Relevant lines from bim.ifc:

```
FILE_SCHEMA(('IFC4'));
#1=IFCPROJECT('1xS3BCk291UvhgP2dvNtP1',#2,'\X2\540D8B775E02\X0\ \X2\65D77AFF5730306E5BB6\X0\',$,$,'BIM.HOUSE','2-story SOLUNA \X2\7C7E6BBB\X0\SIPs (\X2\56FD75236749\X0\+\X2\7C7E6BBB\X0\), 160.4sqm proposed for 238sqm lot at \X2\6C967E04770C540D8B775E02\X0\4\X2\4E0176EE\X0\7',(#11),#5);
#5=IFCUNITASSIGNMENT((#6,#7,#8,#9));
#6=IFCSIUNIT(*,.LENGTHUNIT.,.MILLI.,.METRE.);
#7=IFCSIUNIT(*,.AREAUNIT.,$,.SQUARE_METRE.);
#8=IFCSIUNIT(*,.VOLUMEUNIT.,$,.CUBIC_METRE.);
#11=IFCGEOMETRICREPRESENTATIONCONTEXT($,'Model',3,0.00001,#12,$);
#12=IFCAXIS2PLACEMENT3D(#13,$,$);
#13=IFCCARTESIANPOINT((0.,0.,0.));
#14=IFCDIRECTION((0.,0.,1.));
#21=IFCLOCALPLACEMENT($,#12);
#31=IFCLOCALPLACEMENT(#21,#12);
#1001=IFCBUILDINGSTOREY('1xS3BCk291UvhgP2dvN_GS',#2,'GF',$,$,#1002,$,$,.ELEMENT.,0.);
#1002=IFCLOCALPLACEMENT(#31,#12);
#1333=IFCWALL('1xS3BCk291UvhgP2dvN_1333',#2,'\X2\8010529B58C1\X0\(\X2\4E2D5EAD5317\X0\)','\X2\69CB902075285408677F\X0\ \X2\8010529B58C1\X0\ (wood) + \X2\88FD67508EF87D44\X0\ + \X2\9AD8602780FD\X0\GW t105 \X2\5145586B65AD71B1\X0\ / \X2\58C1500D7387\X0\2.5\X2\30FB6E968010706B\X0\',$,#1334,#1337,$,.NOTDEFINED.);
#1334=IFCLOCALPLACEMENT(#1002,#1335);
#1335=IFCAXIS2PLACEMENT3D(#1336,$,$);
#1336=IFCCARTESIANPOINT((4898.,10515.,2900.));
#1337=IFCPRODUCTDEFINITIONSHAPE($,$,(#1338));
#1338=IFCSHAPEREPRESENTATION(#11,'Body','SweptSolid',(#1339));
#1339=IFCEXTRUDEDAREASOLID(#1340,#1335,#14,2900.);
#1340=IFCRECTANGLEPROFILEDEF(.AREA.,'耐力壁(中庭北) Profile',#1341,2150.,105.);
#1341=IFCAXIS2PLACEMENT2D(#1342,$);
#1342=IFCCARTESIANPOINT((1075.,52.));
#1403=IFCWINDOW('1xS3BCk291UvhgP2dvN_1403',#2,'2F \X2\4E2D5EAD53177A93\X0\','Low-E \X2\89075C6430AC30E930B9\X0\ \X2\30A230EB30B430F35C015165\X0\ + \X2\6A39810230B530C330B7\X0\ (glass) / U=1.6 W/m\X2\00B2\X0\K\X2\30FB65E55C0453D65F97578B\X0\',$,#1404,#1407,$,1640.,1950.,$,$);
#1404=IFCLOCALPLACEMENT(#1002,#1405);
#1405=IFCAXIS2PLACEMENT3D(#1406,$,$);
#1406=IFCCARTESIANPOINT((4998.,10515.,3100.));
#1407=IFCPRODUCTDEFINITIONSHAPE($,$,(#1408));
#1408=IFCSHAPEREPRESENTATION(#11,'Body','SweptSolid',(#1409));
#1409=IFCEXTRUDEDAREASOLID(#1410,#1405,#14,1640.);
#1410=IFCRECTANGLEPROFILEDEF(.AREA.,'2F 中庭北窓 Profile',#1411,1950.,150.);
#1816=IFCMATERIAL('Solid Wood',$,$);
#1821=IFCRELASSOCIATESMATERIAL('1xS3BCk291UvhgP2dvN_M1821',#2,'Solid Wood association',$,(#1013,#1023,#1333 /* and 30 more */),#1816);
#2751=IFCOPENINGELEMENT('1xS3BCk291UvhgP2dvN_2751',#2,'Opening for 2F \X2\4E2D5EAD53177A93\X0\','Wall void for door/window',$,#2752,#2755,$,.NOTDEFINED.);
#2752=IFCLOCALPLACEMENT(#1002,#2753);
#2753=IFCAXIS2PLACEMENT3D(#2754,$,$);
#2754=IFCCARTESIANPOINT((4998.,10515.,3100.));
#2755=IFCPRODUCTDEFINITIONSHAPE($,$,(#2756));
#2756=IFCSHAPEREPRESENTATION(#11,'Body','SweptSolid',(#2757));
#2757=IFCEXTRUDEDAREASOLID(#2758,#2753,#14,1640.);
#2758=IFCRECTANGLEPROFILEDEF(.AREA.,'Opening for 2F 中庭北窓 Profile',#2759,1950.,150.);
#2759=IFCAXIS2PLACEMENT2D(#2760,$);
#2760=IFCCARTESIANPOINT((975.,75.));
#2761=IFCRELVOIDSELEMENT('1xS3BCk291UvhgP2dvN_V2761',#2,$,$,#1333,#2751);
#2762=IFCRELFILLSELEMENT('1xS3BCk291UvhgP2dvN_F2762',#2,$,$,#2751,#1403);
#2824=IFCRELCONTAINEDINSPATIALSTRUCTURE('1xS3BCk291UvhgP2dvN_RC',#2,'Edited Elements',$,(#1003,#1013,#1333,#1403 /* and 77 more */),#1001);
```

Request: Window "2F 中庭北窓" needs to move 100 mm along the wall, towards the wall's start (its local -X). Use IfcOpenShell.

```python
import ifcopenshell
import ifcopenshell.api.geometry
import ifcopenshell.util.placement
import ifcopenshell.util.unit

model = ifcopenshell.open("bim.ifc")
unit_scale = ifcopenshell.util.unit.calculate_unit_scale(model)

window = model.by_guid("1xS3BCk291UvhgP2dvN_1403")
opening = window.FillsVoids[0].RelatingOpeningElement
wall = opening.VoidsElements[0].RelatingBuildingElement

wall_matrix = ifcopenshell.util.placement.get_local_placement(wall.ObjectPlacement)
shift = wall_matrix[:3, 0] * -0.1 / unit_scale
before = ifcopenshell.util.placement.get_local_placement(window.ObjectPlacement)[:3, 3].copy()

# The window is not placed relative to its opening, so move both.
for product in (opening, window):
    matrix = ifcopenshell.util.placement.get_local_placement(product.ObjectPlacement)
    matrix[:3, 3] += shift
    ifcopenshell.api.geometry.edit_object_placement(model, product=product, matrix=matrix, is_si=False)

after = ifcopenshell.util.placement.get_local_placement(window.ObjectPlacement)[:3, 3]
print("window moved by", (after - before).round(3) + 0.0)

model.write("bim_updated.ifc")
```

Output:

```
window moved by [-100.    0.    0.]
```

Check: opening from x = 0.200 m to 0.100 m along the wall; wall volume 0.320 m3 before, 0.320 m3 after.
